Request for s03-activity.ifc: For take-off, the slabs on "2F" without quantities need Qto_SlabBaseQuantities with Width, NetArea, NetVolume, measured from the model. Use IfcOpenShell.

First a look at what the model holds.

```python
import ifcopenshell
import ifcopenshell.util.element
import ifcopenshell.util.unit

model = ifcopenshell.open("s03-activity.ifc")
print(model.schema)
for unit_type in ("LENGTHUNIT", "AREAUNIT", "VOLUMEUNIT"):
    print(unit_type, ifcopenshell.util.unit.calculate_unit_scale(model, unit_type))
storey = next(s for s in model.by_type("IfcBuildingStorey") if s.Name == "2F")
slabs = [e for e in ifcopenshell.util.element.get_decomposition(storey) if e.is_a("IfcSlab")]
for e in sorted(slabs, key=lambda e: e.id()):
    print(e.id(), e.is_a(), e.Name, list(ifcopenshell.util.element.get_psets(e, qtos_only=True)), sep=" | ")
```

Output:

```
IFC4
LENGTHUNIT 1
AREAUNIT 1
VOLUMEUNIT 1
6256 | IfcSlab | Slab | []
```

```python
import ifcopenshell
import ifcopenshell.api.pset
import ifcopenshell.geom
import ifcopenshell.util.element
import ifcopenshell.util.shape
import ifcopenshell.util.unit

model = ifcopenshell.open("s03-activity.ifc")
unit_scale = ifcopenshell.util.unit.calculate_unit_scale(model)
area_scale = ifcopenshell.util.unit.calculate_unit_scale(model, "AREAUNIT")
volume_scale = ifcopenshell.util.unit.calculate_unit_scale(model, "VOLUMEUNIT")
settings = ifcopenshell.geom.settings()

storey = next(s for s in model.by_type("IfcBuildingStorey") if s.Name == "2F")
slabs = [e for e in ifcopenshell.util.element.get_decomposition(storey) if e.is_a("IfcSlab")]

for e in sorted(slabs, key=lambda e: e.id()):
    if ifcopenshell.util.element.get_psets(e, qtos_only=True, should_inherit=False):
        continue
    # Geometry comes back in metres, in the element's own axes.
    shape = ifcopenshell.geom.create_shape(settings, e)
    values = {
        "Width": ifcopenshell.util.shape.get_z(shape.geometry) / unit_scale,
        "NetArea": ifcopenshell.util.shape.get_footprint_area(shape.geometry) / area_scale,
        "NetVolume": ifcopenshell.util.shape.get_volume(shape.geometry) / volume_scale,
    }
    qto = ifcopenshell.api.pset.add_qto(model, product=e, name="Qto_SlabBaseQuantities")
    ifcopenshell.api.pset.edit_qto(model, qto=qto, properties=values)
    print(e.id(), {k: round(v, 3) for k, v in values.items()})

model.write("s03-activity_edited.ifc")
```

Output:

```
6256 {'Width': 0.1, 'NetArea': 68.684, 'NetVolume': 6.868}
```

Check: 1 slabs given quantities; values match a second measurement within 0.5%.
